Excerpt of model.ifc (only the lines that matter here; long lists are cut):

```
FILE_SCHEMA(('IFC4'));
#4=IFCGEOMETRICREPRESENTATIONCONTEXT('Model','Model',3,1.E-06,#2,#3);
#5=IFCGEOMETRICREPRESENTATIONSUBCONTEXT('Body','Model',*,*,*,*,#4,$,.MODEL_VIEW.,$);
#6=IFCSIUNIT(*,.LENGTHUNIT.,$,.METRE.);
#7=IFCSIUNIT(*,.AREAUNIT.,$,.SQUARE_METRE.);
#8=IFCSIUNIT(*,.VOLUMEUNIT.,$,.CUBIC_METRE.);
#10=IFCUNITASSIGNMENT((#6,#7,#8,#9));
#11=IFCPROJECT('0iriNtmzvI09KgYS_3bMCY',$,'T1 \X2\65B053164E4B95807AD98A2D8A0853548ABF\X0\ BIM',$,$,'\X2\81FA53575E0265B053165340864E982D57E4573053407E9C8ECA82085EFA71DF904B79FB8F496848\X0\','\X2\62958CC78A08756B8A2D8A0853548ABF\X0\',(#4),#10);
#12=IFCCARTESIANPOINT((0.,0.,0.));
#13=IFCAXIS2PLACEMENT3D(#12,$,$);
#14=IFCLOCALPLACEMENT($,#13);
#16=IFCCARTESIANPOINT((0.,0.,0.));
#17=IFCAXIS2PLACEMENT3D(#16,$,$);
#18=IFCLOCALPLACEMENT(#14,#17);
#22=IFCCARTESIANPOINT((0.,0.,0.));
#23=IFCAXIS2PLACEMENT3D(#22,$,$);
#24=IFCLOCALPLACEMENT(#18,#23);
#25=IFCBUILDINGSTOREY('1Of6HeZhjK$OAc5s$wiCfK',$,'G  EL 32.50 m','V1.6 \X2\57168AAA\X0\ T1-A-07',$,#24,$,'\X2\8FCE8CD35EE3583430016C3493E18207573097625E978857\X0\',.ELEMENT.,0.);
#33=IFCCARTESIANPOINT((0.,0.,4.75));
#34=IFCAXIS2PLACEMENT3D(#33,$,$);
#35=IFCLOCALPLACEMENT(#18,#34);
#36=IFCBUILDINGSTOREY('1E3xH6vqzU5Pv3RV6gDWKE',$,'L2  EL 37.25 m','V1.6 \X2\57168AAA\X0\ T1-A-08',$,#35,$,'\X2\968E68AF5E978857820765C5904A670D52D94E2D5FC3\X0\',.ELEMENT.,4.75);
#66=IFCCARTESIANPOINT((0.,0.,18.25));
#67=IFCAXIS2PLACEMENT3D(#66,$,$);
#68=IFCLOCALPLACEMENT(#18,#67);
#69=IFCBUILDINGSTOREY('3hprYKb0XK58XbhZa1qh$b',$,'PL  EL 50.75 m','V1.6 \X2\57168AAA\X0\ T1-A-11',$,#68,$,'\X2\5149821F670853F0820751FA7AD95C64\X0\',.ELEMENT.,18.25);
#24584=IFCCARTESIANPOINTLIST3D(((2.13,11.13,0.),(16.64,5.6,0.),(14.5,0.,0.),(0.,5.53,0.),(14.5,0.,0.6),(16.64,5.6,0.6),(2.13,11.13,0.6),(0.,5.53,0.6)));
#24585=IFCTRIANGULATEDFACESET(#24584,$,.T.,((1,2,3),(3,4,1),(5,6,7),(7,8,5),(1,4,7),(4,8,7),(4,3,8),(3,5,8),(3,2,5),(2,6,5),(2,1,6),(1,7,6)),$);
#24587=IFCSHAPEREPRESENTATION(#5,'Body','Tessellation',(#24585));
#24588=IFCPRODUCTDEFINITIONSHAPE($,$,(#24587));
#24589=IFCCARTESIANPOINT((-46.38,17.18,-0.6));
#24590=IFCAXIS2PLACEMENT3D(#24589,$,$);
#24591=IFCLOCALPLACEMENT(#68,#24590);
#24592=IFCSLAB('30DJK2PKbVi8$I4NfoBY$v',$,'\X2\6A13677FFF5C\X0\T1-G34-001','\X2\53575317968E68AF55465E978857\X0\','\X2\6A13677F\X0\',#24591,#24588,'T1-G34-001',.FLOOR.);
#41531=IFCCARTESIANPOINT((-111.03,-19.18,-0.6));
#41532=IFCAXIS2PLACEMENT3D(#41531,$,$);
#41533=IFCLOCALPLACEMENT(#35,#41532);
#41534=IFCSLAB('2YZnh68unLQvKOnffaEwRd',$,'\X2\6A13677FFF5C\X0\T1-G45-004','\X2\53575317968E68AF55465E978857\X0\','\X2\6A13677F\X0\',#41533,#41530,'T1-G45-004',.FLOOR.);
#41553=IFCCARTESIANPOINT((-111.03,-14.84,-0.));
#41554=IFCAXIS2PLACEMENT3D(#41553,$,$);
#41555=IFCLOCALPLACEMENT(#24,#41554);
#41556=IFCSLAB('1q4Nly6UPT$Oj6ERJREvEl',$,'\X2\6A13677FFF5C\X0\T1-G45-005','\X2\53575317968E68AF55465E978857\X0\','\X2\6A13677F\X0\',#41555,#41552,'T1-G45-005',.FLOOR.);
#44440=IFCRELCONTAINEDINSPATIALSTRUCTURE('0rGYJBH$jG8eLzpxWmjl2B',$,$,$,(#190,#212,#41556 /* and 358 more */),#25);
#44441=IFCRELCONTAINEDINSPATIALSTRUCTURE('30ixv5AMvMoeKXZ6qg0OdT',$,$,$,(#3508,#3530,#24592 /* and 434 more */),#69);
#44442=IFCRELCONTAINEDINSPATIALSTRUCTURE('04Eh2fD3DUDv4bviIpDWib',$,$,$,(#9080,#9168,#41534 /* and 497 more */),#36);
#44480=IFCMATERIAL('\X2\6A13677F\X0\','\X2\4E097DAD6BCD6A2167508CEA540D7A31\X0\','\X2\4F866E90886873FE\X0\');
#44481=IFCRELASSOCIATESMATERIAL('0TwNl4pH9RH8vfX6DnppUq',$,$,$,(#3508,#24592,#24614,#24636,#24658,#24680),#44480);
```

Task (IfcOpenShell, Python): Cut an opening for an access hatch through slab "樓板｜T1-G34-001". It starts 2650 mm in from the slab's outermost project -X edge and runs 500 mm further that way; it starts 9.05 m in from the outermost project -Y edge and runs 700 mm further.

```python
import numpy as np
import ifcopenshell
import ifcopenshell.api.feature
import ifcopenshell.api.geometry
import ifcopenshell.api.root
import ifcopenshell.geom
import ifcopenshell.util.placement
import ifcopenshell.util.representation
import ifcopenshell.util.shape
import ifcopenshell.util.unit

model = ifcopenshell.open("model.ifc")
unit_scale = ifcopenshell.util.unit.calculate_unit_scale(model)
settings = ifcopenshell.geom.settings()


def volume(element):
    """Net volume in cubic metres, openings subtracted."""
    shape = ifcopenshell.geom.create_shape(settings, element)
    return ifcopenshell.util.shape.get_volume(shape.geometry)


slab = model.by_guid("30DJK2PKbVi8$I4NfoBY$v")
before = volume(slab)

# Extent in the slab's own axes, in metres. The edges named are its -X and -Y sides.
slab_shape = ifcopenshell.geom.create_shape(settings, slab)
vertices = ifcopenshell.util.shape.get_vertices(slab_shape.geometry)
x_min, y_min, bottom = vertices.min(axis=0)
top = vertices[:, 2].max()

opening = ifcopenshell.api.root.create_entity(model, ifc_class="IfcOpeningElement", name="Access hatch opening", predefined_type="OPENING")
context = ifcopenshell.util.representation.get_context(model, "Model", "Body", "MODEL_VIEW")
width, depth = 0.5, 0.7
outline = [(0.0, 0.0), (width, 0.0), (width, depth), (0.0, depth), (0.0, 0.0)]
# Overshoot both faces by 50 mm so the cut is clean.
shape = ifcopenshell.api.geometry.add_slab_representation(
    model, context=context, depth=top - bottom + 0.1, polyline=outline
)
ifcopenshell.api.geometry.assign_representation(model, product=opening, representation=shape)

matrix = ifcopenshell.util.placement.get_local_placement(slab.ObjectPlacement)
matrix[:, 3] = matrix @ np.append(np.array([x_min + 2.65, y_min + 9.05, bottom - 0.05]) / unit_scale, 1.0)
ifcopenshell.api.geometry.edit_object_placement(model, product=opening, matrix=matrix, is_si=False)
ifcopenshell.api.feature.add_feature(model, feature=opening, element=slab)

after = volume(slab)

print(f"slab volume {before:.3f} -> {after:.3f} m3")

model.write("model_edited.ifc")
```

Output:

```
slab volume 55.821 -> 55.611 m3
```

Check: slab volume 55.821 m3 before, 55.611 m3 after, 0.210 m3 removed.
